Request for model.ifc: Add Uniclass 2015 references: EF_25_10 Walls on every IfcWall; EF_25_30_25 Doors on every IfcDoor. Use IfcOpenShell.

First a look at what the model holds.

```python
import ifcopenshell

model = ifcopenshell.open("model.ifc")
print(model.schema)
print("classifications:", [c.Name for c in model.by_type("IfcClassification")])
for ifc_class in ("IfcDoor", "IfcRoof", "IfcStair", "IfcWall", "IfcWindow"):
    print(ifc_class, len(model.by_type(ifc_class)))
```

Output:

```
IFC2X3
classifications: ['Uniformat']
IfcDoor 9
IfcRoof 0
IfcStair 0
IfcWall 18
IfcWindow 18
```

```python
import ifcopenshell
import ifcopenshell.api.classification

model = ifcopenshell.open("model.ifc")

# IFC2X3 requires Source and Edition and has no link from the project to the system.
system = model.create_entity("IfcClassification", Source="NBS", Edition="2015", Name="Uniclass 2015")

codes = {
    "IfcWall": ("EF_25_10", "Walls"),
    "IfcDoor": ("EF_25_30_25", "Doors"),
}
for ifc_class, (code, name) in codes.items():
    products = model.by_type(ifc_class)
    ifcopenshell.api.classification.add_reference(
        model, products=products, classification=system, identification=code, name=name
    )
    print(code, len(products))

model.write("model_rev.ifc")
```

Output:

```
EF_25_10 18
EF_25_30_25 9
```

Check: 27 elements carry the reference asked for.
